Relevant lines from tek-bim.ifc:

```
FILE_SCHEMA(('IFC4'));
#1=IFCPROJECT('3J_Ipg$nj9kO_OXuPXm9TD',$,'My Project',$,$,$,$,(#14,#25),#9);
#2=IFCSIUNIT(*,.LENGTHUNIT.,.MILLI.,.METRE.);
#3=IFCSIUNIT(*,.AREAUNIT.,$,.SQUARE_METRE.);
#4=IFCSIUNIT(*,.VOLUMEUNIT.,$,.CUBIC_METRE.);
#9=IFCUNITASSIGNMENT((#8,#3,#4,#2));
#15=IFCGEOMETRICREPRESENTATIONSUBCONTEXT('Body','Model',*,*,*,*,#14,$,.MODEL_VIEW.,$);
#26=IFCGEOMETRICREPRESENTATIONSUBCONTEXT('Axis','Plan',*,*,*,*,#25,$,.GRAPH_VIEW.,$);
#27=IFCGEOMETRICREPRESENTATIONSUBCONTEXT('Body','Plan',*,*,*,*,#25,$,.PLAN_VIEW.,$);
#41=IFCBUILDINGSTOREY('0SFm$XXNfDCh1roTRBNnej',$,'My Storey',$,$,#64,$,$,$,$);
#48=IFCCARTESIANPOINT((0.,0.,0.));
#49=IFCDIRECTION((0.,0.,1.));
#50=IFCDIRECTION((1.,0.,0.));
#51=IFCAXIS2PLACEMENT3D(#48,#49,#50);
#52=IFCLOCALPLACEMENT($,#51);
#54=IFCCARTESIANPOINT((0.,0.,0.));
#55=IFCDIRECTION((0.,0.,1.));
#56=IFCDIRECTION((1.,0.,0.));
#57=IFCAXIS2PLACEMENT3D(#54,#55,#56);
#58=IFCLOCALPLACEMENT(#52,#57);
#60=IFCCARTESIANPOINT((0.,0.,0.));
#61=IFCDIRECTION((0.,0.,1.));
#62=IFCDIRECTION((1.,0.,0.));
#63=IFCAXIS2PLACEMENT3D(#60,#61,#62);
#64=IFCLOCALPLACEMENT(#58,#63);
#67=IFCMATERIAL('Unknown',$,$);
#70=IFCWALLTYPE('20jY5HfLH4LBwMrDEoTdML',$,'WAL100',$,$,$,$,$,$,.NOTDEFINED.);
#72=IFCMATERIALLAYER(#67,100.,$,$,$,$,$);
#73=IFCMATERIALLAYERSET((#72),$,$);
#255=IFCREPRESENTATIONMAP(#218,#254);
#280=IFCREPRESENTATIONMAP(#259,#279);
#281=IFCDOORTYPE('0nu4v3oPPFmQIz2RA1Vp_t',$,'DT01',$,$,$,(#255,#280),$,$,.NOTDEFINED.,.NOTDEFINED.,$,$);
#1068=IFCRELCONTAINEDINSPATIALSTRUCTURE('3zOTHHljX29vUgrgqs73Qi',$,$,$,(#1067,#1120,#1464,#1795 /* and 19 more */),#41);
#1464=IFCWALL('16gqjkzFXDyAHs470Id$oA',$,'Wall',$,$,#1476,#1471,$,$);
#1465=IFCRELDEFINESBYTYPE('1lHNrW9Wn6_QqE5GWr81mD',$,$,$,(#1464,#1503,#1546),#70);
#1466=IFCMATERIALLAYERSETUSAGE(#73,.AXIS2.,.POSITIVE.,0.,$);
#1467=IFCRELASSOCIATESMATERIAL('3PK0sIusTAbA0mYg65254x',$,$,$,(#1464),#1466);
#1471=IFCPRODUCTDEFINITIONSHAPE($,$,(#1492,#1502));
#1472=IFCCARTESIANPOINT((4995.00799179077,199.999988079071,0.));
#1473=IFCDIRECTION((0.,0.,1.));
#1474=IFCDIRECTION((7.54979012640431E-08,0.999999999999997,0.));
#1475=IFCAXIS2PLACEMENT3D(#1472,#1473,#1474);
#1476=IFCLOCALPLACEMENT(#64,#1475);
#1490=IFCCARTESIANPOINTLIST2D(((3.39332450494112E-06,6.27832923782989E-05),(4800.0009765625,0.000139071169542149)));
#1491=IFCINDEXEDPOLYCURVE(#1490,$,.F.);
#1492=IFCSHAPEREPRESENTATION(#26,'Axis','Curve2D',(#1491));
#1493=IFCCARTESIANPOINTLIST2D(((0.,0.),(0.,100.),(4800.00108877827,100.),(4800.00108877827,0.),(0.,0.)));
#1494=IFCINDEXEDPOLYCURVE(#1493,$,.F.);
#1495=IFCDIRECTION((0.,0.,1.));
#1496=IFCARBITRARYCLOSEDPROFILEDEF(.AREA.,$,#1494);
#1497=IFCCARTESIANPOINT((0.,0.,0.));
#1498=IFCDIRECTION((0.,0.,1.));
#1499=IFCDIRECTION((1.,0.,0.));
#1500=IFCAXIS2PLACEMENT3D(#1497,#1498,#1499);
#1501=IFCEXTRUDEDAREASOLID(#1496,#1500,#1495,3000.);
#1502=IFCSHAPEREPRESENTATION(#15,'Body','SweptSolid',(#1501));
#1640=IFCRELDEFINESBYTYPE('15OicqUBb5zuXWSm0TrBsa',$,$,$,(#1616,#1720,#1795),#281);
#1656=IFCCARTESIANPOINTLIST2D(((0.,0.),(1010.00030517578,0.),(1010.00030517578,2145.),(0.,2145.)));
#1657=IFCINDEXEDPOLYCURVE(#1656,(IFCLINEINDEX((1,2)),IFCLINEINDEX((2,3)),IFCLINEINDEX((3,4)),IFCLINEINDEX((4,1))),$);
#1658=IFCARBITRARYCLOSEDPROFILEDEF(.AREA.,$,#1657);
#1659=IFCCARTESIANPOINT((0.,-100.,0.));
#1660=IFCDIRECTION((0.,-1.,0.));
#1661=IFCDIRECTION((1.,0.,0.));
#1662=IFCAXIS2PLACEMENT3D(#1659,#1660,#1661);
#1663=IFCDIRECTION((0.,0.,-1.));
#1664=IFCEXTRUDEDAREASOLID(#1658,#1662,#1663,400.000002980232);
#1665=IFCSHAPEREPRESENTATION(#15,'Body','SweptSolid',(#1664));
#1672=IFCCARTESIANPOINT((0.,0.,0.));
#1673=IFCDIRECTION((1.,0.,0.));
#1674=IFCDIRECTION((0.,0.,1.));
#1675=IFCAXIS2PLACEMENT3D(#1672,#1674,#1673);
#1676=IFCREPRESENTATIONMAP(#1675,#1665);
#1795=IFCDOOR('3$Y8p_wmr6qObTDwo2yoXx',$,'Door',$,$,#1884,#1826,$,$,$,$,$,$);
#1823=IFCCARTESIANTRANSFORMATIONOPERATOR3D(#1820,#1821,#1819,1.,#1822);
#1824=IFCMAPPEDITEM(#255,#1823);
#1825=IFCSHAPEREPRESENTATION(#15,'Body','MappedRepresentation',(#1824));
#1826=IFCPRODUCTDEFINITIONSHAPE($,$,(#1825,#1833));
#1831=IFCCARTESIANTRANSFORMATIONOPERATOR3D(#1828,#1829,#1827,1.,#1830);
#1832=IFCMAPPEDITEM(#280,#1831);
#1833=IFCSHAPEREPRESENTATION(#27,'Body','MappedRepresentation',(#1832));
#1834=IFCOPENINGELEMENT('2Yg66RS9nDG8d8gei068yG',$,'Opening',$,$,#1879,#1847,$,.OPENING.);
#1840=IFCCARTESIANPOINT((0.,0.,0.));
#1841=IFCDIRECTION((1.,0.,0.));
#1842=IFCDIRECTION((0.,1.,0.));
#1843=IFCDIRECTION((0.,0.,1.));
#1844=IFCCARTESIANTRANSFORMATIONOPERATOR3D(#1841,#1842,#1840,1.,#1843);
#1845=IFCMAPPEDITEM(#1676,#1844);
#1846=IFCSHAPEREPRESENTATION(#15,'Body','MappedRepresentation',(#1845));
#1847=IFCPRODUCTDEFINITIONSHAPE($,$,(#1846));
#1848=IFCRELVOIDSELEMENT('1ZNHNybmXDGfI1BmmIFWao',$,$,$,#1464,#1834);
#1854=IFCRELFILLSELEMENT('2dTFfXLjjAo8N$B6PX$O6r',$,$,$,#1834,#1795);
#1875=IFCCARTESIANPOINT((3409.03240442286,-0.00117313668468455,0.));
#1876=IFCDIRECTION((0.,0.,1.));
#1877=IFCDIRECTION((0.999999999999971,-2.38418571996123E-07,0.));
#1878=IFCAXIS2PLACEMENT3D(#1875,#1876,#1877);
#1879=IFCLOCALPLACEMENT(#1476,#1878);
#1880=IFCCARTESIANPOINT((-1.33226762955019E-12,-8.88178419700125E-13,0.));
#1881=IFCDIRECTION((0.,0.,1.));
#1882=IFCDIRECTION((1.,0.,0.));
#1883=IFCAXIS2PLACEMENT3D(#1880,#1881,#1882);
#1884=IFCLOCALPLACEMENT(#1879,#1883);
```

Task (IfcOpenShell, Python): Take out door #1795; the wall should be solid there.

```python
import ifcopenshell
import ifcopenshell.api.feature
import ifcopenshell.api.root
import ifcopenshell.geom
import ifcopenshell.util.shape

model = ifcopenshell.open("tek-bim.ifc")
settings = ifcopenshell.geom.settings()


def volume(element):
    """Net volume in cubic metres, openings subtracted."""
    shape = ifcopenshell.geom.create_shape(settings, element)
    return ifcopenshell.util.shape.get_volume(shape.geometry)


door = model.by_guid("3$Y8p_wmr6qObTDwo2yoXx")
opening = door.FillsVoids[0].RelatingOpeningElement
wall = opening.VoidsElements[0].RelatingBuildingElement
before = volume(wall)

ifcopenshell.api.root.remove_product(model, product=door)
ifcopenshell.api.feature.remove_feature(model, feature=opening)

after = volume(wall)

print(f"wall volume {before:.3f} -> {after:.3f} m3")

model.write("tek-bim_v2.ifc")
```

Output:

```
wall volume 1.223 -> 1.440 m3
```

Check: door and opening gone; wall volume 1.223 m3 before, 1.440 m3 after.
